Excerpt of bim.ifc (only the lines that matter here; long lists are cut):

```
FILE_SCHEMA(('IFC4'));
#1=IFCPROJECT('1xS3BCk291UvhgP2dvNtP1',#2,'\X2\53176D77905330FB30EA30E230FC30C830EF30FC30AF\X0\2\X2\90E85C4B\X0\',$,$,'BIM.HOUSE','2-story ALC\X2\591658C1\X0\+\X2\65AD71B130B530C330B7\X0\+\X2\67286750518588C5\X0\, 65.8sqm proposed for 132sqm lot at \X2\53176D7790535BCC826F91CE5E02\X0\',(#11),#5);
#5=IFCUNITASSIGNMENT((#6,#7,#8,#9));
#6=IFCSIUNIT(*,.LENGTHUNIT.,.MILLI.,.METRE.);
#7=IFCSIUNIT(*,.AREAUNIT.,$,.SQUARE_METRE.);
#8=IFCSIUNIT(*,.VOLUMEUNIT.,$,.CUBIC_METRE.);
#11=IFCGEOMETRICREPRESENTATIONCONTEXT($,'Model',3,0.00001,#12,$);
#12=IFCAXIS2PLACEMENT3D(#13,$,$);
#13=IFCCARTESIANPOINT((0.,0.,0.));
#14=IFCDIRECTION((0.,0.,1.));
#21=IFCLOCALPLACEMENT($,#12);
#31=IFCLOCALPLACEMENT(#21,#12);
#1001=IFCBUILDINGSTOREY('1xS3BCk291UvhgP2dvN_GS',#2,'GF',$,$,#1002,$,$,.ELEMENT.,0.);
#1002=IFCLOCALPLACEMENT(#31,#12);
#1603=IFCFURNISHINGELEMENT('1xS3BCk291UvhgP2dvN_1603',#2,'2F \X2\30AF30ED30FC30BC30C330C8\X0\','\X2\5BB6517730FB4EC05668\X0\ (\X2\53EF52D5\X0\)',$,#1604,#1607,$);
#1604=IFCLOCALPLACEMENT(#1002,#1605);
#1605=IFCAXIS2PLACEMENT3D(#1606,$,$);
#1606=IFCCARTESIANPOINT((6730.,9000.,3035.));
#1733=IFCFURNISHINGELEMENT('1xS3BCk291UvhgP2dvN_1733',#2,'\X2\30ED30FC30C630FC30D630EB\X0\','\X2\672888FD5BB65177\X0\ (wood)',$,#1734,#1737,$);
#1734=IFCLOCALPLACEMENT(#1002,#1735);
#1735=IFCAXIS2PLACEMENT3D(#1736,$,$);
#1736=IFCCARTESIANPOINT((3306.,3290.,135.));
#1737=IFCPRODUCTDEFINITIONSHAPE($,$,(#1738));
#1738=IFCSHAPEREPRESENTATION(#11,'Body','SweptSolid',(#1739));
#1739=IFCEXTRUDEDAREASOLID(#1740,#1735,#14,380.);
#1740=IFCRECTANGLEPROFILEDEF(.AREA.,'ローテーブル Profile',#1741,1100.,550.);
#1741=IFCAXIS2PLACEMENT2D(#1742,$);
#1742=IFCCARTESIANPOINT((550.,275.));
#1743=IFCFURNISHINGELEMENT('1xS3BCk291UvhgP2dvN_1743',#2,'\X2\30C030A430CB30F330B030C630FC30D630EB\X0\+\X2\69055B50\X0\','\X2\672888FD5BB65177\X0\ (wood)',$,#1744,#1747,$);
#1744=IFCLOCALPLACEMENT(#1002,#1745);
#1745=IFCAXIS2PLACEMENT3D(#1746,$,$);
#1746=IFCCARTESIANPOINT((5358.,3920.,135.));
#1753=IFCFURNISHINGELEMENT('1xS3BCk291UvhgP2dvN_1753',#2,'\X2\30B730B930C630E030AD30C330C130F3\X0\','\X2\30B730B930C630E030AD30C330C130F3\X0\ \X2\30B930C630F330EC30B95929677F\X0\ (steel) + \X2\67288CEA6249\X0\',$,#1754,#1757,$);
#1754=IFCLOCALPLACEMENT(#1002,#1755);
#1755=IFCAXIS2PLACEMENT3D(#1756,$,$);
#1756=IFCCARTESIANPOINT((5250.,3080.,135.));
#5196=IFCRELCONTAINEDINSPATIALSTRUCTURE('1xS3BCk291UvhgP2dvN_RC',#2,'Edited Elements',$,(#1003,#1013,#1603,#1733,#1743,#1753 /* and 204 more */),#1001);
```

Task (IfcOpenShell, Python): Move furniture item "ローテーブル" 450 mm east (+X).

```python
import ifcopenshell
import ifcopenshell.api.geometry
import ifcopenshell.util.placement

model = ifcopenshell.open("bim.ifc")

item = model.by_guid("1xS3BCk291UvhgP2dvN_1733")
matrix = ifcopenshell.util.placement.get_local_placement(item.ObjectPlacement)
matrix[0, 3] += 450.0
ifcopenshell.api.geometry.edit_object_placement(model, product=item, matrix=matrix, is_si=False)

print(ifcopenshell.util.placement.get_local_placement(item.ObjectPlacement).round(3) + 0.0)

model.write("bim_rev.ifc")
```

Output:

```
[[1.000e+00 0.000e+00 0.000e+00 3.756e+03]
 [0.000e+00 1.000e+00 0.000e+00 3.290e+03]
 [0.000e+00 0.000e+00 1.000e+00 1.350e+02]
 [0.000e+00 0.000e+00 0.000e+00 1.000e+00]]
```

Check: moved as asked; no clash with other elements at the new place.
